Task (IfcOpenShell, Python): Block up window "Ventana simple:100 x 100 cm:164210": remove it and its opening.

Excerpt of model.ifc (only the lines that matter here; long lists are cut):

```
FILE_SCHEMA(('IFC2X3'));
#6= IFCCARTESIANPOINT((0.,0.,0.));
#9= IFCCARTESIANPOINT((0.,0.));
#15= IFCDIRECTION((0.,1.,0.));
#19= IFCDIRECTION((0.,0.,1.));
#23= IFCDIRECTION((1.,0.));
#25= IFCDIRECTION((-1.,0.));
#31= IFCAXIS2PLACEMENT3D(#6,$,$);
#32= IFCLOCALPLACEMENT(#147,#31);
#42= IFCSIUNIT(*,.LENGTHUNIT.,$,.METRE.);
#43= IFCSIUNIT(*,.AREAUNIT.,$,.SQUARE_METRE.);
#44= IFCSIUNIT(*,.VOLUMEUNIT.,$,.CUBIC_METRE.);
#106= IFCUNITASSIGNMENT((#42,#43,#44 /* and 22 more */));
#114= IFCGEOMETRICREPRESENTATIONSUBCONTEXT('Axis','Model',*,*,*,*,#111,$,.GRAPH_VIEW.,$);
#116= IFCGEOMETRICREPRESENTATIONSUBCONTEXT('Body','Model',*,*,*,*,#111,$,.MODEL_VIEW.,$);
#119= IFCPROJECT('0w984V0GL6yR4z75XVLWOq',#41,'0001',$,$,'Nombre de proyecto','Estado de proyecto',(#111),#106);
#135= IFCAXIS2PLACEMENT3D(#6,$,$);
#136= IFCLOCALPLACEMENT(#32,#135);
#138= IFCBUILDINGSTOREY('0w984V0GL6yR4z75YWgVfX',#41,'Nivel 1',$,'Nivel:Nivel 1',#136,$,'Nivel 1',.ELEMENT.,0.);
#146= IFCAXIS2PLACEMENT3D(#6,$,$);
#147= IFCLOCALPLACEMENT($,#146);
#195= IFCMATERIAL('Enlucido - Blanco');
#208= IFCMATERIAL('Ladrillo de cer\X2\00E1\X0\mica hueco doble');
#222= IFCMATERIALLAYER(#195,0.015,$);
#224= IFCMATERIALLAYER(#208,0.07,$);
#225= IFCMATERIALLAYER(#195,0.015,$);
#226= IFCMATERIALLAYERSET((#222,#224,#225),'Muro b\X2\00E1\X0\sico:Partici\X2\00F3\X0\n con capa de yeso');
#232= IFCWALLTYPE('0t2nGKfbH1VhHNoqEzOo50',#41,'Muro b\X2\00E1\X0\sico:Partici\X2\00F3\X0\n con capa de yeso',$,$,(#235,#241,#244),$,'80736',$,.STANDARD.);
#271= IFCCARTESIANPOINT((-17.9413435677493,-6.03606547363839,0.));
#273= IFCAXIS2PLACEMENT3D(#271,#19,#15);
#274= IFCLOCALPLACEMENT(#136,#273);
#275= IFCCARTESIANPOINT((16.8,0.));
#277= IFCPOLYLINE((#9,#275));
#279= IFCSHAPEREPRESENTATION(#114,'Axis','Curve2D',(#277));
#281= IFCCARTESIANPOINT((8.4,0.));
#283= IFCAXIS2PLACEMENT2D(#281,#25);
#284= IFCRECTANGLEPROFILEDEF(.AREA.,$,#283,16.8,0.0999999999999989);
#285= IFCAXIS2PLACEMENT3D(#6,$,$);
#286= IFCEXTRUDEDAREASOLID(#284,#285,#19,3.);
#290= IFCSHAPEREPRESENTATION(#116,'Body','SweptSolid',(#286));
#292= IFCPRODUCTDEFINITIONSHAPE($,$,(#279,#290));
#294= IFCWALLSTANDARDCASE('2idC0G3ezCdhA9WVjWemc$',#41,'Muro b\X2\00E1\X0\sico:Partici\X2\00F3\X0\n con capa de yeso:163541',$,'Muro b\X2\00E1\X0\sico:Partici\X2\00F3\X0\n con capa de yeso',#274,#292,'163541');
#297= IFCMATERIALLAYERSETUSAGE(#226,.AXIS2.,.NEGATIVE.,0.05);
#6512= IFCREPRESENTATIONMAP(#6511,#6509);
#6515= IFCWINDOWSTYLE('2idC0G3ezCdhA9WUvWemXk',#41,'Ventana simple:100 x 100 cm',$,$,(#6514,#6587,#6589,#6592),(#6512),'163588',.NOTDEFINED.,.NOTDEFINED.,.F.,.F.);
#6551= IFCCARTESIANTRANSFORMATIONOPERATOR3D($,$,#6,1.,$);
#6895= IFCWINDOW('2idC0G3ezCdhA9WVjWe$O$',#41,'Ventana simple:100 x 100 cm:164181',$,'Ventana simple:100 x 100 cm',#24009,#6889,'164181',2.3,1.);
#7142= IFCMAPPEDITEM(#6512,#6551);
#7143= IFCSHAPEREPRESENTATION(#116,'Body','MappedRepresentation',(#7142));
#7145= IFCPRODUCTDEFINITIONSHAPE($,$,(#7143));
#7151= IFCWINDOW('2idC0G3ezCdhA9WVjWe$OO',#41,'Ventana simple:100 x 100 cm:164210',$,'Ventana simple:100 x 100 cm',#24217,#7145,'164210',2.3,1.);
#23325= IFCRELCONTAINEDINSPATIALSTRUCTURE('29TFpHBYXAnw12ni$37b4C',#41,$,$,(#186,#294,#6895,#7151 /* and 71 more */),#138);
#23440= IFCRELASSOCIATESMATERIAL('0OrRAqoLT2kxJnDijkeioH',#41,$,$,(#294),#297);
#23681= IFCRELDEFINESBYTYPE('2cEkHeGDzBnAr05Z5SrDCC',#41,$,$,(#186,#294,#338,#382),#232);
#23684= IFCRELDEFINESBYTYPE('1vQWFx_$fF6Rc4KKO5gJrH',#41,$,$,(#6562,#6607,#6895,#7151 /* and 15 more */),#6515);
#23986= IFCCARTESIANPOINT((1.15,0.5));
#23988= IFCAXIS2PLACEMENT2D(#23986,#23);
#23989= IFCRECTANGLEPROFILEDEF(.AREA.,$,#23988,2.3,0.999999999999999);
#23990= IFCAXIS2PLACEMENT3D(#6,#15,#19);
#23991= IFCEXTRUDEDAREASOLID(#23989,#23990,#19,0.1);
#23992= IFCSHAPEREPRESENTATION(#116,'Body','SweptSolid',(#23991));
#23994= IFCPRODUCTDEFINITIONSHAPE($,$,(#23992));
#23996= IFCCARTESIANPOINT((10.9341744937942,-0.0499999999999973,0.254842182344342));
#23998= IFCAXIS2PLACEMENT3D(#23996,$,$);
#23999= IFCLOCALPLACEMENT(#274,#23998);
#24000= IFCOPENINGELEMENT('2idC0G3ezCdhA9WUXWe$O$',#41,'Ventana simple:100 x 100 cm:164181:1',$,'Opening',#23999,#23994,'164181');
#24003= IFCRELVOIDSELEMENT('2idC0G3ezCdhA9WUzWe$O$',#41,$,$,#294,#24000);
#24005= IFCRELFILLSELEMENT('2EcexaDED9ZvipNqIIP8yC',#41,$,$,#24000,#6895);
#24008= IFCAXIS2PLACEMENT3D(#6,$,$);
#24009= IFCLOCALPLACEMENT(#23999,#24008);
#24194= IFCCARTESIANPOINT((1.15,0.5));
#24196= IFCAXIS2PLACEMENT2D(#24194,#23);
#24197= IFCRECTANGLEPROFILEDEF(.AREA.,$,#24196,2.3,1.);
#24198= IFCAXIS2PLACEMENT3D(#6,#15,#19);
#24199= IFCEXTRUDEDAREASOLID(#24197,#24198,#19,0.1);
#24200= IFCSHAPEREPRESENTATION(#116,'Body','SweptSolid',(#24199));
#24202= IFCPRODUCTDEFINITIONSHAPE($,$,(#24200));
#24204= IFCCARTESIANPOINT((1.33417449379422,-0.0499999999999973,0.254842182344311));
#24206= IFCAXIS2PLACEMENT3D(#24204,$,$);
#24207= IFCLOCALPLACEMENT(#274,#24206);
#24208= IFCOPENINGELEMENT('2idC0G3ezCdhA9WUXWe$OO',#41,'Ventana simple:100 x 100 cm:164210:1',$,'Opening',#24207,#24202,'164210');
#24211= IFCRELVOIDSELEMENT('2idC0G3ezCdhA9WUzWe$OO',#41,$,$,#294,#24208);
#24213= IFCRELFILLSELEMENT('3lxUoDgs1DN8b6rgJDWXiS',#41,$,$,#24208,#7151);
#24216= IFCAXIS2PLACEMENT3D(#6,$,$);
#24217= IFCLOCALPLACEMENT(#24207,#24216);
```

```python
import ifcopenshell
import ifcopenshell.api.feature
import ifcopenshell.api.root
import ifcopenshell.geom
import ifcopenshell.util.shape

model = ifcopenshell.open("model.ifc")
settings = ifcopenshell.geom.settings()


def volume(element):
    """Net volume in cubic metres, openings subtracted."""
    shape = ifcopenshell.geom.create_shape(settings, element)
    return ifcopenshell.util.shape.get_volume(shape.geometry)


window = model.by_guid("2idC0G3ezCdhA9WVjWe$OO")
opening = window.FillsVoids[0].RelatingOpeningElement
wall = opening.VoidsElements[0].RelatingBuildingElement
before = volume(wall)

ifcopenshell.api.root.remove_product(model, product=window)
ifcopenshell.api.feature.remove_feature(model, feature=opening)

after = volume(wall)

print(f"wall volume {before:.3f} -> {after:.3f} m3")

model.write("model_updated.ifc")
```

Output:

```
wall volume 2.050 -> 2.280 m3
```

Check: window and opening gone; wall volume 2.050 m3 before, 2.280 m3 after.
